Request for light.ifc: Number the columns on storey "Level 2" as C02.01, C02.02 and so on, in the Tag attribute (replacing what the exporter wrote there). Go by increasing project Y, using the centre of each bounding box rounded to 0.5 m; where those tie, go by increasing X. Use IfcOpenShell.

First a look at what the model holds.

```python
import ifcopenshell
import ifcopenshell.util.element
import ifcopenshell.util.placement

model = ifcopenshell.open("light.ifc")
print(model.schema)
storey = next(s for s in model.by_type("IfcBuildingStorey") if s.Name == "Level 2")
columns = [e for e in ifcopenshell.util.element.get_decomposition(storey) if e.is_a("IfcColumn")]
for e in sorted(columns, key=lambda e: e.id()):
    origin = ifcopenshell.util.placement.get_local_placement(e.ObjectPlacement)[:3, 3]
    print(e.id(), e.Tag, e.Name, origin.round(2) + 0.0, sep=" | ")
```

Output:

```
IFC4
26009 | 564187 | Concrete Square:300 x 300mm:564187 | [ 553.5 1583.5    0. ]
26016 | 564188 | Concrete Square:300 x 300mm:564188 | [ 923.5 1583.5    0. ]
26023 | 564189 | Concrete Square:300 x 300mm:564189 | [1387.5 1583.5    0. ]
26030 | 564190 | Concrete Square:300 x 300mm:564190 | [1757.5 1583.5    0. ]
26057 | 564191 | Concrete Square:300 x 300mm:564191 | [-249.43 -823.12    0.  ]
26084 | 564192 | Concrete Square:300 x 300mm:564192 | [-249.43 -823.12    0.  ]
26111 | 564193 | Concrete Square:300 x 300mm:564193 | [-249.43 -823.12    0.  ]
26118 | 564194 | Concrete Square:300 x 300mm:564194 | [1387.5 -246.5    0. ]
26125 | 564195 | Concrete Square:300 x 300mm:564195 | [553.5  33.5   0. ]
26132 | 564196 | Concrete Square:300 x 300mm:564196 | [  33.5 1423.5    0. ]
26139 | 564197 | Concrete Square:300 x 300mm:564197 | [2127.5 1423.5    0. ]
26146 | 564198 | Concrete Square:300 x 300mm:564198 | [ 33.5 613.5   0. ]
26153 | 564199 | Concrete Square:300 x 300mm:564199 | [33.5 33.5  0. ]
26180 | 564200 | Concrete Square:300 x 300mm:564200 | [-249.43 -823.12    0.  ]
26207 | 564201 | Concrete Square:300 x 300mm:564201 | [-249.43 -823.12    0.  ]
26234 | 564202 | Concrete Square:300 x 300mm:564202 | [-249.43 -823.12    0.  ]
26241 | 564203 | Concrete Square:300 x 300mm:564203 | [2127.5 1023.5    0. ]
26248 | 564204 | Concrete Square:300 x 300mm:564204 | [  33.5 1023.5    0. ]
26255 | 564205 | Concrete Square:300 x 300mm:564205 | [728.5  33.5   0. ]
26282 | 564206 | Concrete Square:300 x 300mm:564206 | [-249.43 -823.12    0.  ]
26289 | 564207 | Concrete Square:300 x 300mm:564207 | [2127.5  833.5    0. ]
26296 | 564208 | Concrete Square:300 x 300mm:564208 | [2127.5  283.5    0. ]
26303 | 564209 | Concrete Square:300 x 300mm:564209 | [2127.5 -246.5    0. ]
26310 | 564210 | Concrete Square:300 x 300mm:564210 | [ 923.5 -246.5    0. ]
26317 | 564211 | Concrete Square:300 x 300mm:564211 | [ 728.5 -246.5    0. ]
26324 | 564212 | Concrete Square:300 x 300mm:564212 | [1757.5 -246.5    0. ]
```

```python
import ifcopenshell
import ifcopenshell.geom
import ifcopenshell.util.element
import ifcopenshell.util.shape

model = ifcopenshell.open("light.ifc")
settings = ifcopenshell.geom.settings()
settings.set("use-world-coords", True)


def centre(element):
    shape = ifcopenshell.geom.create_shape(settings, element)
    return ifcopenshell.util.shape.get_bbox_centroid(shape.geometry)


storey = next(s for s in model.by_type("IfcBuildingStorey") if s.Name == "Level 2")
columns = [e for e in ifcopenshell.util.element.get_decomposition(storey) if e.is_a("IfcColumn")]

# Insertion points can sit at a corner or the storey origin, so sort by the geometry (in metres).
centres = {e: centre(e) for e in columns}
columns.sort(key=lambda e: (round(centres[e][1] / 0.5), centres[e][0]))

for i, e in enumerate(columns, start=1):
    number = f"C02.{i:02d}"
    e.Tag = number
    print(e.id(), number)

model.write("light_updated.ifc")
```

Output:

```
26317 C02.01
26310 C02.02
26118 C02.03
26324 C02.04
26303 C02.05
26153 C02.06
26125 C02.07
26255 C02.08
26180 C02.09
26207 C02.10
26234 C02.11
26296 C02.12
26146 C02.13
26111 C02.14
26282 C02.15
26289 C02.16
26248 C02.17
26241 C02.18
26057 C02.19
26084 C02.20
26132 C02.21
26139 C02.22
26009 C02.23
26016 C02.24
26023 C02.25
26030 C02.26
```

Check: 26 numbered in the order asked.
